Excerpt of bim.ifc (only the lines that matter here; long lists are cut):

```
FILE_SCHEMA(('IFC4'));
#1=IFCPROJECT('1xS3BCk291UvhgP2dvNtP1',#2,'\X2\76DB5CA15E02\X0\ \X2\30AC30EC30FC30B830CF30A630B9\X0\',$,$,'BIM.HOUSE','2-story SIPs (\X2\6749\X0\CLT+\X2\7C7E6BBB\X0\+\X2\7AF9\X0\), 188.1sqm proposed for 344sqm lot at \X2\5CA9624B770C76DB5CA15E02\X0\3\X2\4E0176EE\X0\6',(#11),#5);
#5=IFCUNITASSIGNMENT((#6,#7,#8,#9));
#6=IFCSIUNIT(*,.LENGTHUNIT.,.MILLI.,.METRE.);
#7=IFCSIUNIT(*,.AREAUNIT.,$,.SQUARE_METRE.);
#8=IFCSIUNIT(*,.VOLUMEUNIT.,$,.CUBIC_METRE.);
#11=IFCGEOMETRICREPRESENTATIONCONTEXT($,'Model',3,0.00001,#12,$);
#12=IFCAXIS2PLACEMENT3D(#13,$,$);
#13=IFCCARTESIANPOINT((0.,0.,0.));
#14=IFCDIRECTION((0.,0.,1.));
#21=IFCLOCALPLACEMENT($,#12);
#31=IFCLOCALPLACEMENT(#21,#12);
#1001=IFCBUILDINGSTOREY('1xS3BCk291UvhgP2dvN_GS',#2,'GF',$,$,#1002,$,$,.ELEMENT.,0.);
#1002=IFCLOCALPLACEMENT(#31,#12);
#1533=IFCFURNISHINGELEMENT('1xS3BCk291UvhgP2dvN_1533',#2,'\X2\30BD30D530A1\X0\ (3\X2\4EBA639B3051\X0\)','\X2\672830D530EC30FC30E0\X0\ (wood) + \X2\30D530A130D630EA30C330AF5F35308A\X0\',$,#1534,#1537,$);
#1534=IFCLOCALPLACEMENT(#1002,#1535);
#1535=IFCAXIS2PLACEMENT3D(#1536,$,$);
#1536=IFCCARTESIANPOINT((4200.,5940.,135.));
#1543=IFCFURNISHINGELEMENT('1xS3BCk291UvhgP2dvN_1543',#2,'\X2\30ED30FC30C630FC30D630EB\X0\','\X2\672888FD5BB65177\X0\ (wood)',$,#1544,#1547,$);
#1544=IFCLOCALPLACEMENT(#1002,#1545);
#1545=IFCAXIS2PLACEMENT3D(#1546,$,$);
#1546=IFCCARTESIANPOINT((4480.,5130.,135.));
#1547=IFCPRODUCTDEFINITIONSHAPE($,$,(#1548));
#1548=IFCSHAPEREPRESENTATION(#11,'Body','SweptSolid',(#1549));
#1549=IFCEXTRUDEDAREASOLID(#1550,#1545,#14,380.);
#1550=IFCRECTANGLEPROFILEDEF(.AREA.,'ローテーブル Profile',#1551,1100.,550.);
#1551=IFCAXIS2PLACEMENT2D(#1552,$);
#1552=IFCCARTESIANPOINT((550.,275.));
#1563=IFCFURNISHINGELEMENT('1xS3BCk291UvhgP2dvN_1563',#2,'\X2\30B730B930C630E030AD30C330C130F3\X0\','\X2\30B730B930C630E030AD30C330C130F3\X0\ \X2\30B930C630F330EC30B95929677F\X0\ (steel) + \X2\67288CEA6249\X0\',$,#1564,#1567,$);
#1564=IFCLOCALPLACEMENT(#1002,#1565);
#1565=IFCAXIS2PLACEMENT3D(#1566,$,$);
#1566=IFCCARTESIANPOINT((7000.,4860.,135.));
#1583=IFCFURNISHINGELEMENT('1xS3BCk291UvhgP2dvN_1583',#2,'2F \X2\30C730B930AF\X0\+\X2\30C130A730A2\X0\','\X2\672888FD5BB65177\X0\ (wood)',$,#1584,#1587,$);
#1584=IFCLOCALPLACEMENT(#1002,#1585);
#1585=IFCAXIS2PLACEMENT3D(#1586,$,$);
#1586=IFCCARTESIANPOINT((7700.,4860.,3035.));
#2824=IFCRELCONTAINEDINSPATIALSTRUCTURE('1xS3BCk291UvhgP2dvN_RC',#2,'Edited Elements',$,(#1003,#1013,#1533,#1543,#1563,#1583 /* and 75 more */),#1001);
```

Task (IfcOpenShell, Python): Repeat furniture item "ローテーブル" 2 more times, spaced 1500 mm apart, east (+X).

```python
import numpy as np
import ifcopenshell
import ifcopenshell.api.geometry
import ifcopenshell.api.root
import ifcopenshell.util.element
import ifcopenshell.util.placement
import ifcopenshell.util.unit

model = ifcopenshell.open("bim.ifc")
unit_scale = ifcopenshell.util.unit.calculate_unit_scale(model)


def reuse_history(source, copy):
    """copy_class also copies each property set's owner history, people and application; keep the originals."""
    for rel in copy.IsDefinedBy:
        if rel.is_a("IfcRelDefinesByProperties") and (history := rel.RelatingPropertyDefinition.OwnerHistory):
            rel.RelatingPropertyDefinition.OwnerHistory = source.OwnerHistory
            ifcopenshell.util.element.remove_deep2(model, history)


source = model.by_guid("1xS3BCk291UvhgP2dvN_1543")
base = ifcopenshell.util.placement.get_local_placement(source.ObjectPlacement)
step = np.array([1.0, 0.0, 0.0]) * 1.5 / unit_scale

for i in range(1, 3):
    copy = ifcopenshell.api.root.copy_class(model, product=source)
    copy.Representation = ifcopenshell.util.element.copy_deep(
        model, source.Representation, exclude=["IfcGeometricRepresentationContext", "IfcRepresentationMap"]
    )
    reuse_history(source, copy)
    matrix = base.copy()
    matrix[:3, 3] += i * step
    print("added at", matrix[:3, 3].round(3) + 0.0)
    ifcopenshell.api.geometry.edit_object_placement(model, product=copy, matrix=matrix, is_si=False)

model.write("bim_rev.ifc")
```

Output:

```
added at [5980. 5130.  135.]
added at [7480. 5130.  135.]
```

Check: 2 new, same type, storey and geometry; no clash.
